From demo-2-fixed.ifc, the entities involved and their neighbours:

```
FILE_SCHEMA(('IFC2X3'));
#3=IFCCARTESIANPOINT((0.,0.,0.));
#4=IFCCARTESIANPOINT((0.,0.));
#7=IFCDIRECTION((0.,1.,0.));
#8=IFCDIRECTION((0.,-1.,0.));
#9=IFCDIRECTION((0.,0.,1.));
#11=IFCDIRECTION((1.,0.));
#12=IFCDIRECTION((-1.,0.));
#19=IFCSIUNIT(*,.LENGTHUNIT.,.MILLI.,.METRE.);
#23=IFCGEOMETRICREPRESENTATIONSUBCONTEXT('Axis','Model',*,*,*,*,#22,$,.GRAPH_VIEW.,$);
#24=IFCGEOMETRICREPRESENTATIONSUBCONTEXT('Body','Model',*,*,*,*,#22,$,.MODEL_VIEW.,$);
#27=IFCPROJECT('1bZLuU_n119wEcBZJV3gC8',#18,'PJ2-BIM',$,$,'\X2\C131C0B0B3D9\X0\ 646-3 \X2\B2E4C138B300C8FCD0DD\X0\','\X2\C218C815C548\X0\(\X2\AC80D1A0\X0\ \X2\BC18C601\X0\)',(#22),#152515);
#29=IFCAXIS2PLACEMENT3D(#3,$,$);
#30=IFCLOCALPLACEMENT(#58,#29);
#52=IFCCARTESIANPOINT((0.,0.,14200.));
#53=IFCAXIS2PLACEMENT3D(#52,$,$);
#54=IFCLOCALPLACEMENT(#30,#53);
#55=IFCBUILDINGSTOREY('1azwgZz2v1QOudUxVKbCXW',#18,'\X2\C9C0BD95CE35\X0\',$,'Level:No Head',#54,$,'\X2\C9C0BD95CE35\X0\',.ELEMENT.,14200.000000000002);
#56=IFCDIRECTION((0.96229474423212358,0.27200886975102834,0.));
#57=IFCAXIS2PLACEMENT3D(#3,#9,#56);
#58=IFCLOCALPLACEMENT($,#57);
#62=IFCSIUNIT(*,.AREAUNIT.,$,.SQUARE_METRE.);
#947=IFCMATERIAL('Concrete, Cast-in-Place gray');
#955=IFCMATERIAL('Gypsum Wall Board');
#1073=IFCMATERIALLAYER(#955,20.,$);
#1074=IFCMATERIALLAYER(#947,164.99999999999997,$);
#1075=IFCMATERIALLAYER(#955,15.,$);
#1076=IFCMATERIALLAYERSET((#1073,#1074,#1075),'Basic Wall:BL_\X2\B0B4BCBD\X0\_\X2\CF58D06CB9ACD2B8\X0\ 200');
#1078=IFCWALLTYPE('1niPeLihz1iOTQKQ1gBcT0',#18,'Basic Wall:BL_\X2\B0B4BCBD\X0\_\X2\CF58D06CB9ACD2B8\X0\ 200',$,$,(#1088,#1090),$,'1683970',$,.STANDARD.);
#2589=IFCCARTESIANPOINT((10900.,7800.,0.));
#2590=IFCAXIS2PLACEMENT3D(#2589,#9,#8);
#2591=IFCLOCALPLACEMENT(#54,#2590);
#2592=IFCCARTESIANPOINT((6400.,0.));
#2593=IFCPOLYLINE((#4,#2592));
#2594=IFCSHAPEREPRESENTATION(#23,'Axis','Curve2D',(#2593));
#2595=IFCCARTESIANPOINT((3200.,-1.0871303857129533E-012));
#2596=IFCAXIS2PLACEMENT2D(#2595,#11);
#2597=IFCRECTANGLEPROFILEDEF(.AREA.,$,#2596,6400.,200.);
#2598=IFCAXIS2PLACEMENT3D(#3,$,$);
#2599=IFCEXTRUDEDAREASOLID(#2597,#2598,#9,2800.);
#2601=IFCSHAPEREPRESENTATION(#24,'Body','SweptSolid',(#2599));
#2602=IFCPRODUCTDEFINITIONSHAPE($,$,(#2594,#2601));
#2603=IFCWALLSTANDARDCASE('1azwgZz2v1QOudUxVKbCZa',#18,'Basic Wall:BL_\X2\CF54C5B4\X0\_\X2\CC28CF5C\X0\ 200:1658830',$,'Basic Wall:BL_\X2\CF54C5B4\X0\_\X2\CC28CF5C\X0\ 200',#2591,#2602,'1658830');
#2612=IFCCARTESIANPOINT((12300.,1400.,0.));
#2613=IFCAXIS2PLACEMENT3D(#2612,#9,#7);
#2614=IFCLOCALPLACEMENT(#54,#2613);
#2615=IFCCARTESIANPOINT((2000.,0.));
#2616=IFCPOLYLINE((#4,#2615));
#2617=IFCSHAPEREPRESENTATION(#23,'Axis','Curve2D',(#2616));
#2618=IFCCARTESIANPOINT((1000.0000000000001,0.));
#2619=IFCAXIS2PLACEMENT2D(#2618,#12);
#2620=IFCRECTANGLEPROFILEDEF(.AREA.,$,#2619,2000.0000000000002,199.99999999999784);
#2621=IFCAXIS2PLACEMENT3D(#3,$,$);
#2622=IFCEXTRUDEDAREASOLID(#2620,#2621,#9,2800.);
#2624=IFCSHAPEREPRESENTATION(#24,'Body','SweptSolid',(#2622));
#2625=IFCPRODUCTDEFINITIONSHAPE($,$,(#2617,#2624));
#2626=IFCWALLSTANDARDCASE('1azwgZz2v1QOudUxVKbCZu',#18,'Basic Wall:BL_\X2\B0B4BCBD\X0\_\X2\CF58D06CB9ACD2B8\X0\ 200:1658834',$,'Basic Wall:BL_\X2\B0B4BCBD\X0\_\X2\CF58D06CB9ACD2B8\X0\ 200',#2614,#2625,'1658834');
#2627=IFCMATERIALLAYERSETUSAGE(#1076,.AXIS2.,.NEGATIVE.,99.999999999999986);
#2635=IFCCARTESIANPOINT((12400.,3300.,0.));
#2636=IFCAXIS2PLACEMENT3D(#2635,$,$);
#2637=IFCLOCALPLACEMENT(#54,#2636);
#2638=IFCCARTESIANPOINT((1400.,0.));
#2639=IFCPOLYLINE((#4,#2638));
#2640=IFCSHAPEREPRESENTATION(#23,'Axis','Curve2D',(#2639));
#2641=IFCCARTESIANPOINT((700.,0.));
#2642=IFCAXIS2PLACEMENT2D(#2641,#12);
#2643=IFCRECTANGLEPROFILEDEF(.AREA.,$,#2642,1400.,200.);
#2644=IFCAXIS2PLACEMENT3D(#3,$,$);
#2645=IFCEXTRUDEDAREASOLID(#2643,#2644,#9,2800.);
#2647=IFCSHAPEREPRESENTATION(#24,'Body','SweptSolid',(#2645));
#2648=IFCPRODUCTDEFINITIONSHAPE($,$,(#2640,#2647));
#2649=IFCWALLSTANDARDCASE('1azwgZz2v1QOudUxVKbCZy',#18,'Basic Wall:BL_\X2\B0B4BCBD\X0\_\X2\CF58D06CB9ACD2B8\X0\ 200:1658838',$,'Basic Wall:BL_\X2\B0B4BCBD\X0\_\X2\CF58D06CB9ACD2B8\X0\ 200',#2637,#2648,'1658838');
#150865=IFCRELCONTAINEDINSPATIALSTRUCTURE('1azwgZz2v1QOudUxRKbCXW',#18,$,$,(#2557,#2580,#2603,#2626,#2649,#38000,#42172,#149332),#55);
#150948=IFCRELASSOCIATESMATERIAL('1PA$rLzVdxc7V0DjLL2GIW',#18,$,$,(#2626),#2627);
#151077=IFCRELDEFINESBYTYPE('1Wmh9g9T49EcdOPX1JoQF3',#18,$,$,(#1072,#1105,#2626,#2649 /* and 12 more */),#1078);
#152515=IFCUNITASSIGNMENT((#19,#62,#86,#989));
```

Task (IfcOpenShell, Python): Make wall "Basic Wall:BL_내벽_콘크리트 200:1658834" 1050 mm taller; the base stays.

```python
import ifcopenshell
import ifcopenshell.geom
import ifcopenshell.util.representation
import ifcopenshell.util.shape
import ifcopenshell.util.unit

model = ifcopenshell.open("demo-2-fixed.ifc")
unit_scale = ifcopenshell.util.unit.calculate_unit_scale(model)
settings = ifcopenshell.geom.settings()


def volume(element):
    """Net volume in cubic metres, openings subtracted."""
    shape = ifcopenshell.geom.create_shape(settings, element)
    return ifcopenshell.util.shape.get_volume(shape.geometry)


wall = model.by_guid("1azwgZz2v1QOudUxVKbCZu")
before = volume(wall)

body = ifcopenshell.util.representation.get_representation(wall, "Model", "Body")
solid = body.Items[0]
old_height = solid.Depth
solid.Depth += 1.05 / unit_scale
after = volume(wall)

print(f"height {old_height:g} -> {solid.Depth:g}, volume {before:.3f} -> {after:.3f} m3")

model.write("demo-2-fixed_v2.ifc")
```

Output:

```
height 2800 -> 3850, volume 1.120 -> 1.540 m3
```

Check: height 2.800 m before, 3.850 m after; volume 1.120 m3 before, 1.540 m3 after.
